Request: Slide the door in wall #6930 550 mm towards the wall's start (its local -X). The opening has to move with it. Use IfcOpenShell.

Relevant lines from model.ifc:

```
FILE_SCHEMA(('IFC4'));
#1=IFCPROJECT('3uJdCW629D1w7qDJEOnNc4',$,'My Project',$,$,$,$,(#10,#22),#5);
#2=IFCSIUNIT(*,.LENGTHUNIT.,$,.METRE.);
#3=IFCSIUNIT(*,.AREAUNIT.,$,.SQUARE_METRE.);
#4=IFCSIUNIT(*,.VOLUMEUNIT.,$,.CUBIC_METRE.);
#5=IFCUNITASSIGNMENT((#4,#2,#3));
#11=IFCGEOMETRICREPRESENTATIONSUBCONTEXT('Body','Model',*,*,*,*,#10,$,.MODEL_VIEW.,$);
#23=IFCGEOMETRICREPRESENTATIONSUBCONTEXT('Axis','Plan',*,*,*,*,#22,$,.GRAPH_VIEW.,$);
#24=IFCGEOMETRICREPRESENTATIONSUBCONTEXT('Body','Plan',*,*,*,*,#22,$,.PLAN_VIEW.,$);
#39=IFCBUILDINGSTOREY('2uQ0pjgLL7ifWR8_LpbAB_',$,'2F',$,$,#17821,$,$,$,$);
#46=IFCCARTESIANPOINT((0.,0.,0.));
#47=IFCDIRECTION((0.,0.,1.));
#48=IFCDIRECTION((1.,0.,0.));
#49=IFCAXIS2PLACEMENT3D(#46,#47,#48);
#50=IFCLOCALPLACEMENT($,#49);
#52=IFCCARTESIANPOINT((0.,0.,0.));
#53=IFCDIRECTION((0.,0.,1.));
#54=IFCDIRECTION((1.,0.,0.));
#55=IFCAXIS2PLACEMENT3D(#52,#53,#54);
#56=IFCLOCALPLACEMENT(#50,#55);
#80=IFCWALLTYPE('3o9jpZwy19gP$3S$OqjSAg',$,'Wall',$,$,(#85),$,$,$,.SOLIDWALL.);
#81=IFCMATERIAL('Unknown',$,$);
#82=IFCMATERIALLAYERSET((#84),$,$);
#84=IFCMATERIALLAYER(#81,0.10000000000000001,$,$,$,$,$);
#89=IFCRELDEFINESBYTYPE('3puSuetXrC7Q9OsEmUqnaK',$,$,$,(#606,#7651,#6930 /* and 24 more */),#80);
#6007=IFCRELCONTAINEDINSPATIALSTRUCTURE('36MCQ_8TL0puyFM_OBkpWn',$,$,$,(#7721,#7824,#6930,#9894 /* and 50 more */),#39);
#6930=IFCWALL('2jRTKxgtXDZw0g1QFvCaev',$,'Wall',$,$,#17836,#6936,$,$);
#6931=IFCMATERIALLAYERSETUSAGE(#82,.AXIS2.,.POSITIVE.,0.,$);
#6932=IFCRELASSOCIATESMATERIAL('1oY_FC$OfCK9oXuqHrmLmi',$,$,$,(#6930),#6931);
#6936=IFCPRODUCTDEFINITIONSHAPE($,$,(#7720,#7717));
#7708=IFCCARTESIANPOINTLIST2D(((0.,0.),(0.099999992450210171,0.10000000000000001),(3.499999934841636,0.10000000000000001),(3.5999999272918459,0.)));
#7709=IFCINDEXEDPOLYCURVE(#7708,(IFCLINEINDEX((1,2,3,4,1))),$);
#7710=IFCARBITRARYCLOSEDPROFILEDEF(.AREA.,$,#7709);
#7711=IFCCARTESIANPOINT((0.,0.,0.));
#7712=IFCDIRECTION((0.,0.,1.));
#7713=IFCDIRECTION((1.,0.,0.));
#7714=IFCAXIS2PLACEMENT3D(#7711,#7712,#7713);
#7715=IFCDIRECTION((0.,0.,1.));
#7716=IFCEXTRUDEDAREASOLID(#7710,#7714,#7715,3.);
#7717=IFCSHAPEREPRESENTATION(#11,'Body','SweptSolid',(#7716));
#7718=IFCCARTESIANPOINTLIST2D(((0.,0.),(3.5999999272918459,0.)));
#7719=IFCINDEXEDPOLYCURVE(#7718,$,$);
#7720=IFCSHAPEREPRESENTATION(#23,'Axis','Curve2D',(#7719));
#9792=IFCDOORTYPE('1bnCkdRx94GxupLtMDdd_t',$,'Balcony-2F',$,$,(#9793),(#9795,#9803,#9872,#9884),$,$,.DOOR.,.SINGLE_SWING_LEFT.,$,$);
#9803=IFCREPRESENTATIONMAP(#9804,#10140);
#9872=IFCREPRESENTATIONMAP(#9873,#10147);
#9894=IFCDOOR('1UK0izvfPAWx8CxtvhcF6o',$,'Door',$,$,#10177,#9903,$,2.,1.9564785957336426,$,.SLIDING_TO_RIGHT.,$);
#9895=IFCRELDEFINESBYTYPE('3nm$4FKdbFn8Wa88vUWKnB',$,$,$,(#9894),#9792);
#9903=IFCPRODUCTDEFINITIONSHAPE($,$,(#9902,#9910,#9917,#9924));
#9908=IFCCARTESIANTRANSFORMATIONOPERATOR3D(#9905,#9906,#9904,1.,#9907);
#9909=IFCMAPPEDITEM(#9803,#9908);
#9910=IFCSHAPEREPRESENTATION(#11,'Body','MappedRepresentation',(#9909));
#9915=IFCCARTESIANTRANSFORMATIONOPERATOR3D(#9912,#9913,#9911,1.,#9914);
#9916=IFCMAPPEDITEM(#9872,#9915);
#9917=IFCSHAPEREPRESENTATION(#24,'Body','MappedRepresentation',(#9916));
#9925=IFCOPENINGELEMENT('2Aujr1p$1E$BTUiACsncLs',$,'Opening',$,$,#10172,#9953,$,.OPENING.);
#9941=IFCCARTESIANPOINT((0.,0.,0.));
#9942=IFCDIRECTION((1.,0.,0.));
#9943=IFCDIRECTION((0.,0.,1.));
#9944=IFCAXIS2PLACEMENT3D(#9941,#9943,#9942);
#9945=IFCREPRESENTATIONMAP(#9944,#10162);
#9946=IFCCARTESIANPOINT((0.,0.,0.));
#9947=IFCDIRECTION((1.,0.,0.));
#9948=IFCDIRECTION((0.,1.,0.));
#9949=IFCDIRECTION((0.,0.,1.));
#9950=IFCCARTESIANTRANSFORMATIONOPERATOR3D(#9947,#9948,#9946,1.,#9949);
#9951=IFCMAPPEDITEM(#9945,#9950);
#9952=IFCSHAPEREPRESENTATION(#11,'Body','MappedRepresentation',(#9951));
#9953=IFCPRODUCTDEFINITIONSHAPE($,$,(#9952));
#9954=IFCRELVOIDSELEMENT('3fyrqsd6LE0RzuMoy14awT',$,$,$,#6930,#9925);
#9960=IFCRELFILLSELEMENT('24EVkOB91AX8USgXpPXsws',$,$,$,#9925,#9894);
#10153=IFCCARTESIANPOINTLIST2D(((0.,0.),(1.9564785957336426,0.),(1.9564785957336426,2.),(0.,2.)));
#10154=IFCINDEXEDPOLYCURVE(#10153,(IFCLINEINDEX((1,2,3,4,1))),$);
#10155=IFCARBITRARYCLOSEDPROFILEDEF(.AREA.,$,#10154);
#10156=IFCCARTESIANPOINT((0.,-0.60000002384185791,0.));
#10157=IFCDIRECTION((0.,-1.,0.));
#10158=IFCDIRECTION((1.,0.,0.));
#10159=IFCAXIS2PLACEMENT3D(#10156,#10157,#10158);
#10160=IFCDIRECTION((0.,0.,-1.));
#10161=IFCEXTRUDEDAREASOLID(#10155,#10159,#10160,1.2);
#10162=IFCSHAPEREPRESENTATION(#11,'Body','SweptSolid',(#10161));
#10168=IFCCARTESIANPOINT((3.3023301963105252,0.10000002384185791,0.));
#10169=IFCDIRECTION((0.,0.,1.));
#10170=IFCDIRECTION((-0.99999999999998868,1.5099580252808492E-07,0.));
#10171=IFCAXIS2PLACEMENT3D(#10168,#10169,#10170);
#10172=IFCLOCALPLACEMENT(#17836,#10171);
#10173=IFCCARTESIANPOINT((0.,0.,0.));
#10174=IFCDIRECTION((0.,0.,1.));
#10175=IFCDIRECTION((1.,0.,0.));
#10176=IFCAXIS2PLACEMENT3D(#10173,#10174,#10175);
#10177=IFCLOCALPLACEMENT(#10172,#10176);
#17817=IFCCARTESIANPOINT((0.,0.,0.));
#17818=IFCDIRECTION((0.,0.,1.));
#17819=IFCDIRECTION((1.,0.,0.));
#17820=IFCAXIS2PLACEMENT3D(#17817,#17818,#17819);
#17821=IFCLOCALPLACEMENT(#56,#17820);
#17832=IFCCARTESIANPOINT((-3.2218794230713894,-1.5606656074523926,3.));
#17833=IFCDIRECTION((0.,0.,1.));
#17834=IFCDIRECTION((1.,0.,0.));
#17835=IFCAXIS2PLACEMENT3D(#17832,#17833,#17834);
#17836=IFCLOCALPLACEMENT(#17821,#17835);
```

```python
import ifcopenshell
import ifcopenshell.api.geometry
import ifcopenshell.util.placement
import ifcopenshell.util.unit

model = ifcopenshell.open("model.ifc")
unit_scale = ifcopenshell.util.unit.calculate_unit_scale(model)

door = model.by_id(9894)
opening = door.FillsVoids[0].RelatingOpeningElement
wall = opening.VoidsElements[0].RelatingBuildingElement

wall_matrix = ifcopenshell.util.placement.get_local_placement(wall.ObjectPlacement)
shift = wall_matrix[:3, 0] * -0.55 / unit_scale
before = ifcopenshell.util.placement.get_local_placement(door.ObjectPlacement)[:3, 3].copy()

# The door is placed relative to its opening, so it follows when the opening moves.
matrix = ifcopenshell.util.placement.get_local_placement(opening.ObjectPlacement)
matrix[:3, 3] += shift
ifcopenshell.api.geometry.edit_object_placement(
    model, product=opening, matrix=matrix, is_si=False, should_transform_children=True
)

after = ifcopenshell.util.placement.get_local_placement(door.ObjectPlacement)[:3, 3]
print("door moved by", (after - before).round(3) + 0.0)

model.write("model_rev.ifc")
```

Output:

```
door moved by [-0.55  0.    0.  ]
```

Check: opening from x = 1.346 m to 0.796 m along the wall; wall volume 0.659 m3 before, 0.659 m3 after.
